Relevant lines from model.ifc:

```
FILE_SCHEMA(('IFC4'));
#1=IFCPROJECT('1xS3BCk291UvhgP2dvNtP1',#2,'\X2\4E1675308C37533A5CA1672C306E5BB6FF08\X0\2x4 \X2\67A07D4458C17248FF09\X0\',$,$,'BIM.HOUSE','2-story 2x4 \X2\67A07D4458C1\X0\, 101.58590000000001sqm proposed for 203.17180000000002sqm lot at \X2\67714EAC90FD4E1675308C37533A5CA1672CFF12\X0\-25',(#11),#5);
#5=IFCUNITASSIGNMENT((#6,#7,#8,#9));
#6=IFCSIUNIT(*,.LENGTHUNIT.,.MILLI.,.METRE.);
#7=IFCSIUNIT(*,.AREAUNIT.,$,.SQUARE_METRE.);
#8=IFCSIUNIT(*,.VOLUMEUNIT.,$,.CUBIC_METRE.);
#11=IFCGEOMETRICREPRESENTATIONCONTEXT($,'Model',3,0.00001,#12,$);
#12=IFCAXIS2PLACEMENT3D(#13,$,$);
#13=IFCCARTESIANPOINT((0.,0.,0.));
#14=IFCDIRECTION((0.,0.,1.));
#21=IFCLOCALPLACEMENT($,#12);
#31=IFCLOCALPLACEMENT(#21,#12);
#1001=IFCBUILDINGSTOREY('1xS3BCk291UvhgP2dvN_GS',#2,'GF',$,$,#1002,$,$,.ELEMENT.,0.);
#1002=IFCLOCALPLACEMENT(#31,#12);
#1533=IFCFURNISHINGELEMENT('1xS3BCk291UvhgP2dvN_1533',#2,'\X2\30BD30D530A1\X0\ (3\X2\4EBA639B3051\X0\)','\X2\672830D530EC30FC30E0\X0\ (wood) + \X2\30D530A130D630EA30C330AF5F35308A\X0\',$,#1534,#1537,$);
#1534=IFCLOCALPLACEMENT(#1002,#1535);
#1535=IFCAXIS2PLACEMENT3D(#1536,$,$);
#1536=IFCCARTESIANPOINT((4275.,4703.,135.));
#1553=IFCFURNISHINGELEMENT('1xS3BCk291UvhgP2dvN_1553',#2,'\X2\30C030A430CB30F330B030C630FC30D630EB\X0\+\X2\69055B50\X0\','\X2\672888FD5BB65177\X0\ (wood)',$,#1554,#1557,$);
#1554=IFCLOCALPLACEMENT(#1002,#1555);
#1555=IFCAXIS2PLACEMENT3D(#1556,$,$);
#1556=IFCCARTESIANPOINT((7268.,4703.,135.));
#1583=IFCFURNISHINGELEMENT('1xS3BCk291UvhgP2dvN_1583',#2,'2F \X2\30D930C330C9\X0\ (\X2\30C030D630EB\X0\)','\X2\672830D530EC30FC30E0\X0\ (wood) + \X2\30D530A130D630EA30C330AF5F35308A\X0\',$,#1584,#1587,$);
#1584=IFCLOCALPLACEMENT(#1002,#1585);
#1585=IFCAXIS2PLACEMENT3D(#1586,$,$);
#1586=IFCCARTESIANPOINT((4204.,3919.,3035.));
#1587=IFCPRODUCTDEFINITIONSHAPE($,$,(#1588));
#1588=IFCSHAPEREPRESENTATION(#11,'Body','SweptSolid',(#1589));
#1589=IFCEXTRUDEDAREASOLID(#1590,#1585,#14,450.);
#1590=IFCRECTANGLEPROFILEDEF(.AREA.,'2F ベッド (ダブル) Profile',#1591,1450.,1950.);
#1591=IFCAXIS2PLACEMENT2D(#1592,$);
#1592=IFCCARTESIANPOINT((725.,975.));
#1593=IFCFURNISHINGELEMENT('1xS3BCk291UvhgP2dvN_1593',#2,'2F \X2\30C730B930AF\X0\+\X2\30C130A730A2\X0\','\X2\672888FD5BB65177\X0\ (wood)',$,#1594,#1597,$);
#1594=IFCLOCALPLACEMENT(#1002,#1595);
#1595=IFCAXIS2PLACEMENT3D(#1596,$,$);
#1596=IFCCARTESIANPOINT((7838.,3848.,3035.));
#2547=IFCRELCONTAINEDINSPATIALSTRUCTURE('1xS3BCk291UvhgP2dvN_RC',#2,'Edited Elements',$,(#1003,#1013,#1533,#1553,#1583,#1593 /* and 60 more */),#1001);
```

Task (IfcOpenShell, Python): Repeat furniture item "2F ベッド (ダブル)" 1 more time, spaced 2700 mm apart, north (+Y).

```python
import numpy as np
import ifcopenshell
import ifcopenshell.api.geometry
import ifcopenshell.api.root
import ifcopenshell.util.element
import ifcopenshell.util.placement
import ifcopenshell.util.unit

model = ifcopenshell.open("model.ifc")
unit_scale = ifcopenshell.util.unit.calculate_unit_scale(model)


def reuse_history(source, copy):
    """copy_class also copies each property set's owner history, people and application; keep the originals."""
    for rel in copy.IsDefinedBy:
        if rel.is_a("IfcRelDefinesByProperties") and (history := rel.RelatingPropertyDefinition.OwnerHistory):
            rel.RelatingPropertyDefinition.OwnerHistory = source.OwnerHistory
            ifcopenshell.util.element.remove_deep2(model, history)


source = model.by_guid("1xS3BCk291UvhgP2dvN_1583")
base = ifcopenshell.util.placement.get_local_placement(source.ObjectPlacement)
step = np.array([0.0, 1.0, 0.0]) * 2.7 / unit_scale

for i in range(1, 2):
    copy = ifcopenshell.api.root.copy_class(model, product=source)
    copy.Representation = ifcopenshell.util.element.copy_deep(
        model, source.Representation, exclude=["IfcGeometricRepresentationContext", "IfcRepresentationMap"]
    )
    reuse_history(source, copy)
    matrix = base.copy()
    matrix[:3, 3] += i * step
    print("added at", matrix[:3, 3].round(3) + 0.0)
    ifcopenshell.api.geometry.edit_object_placement(model, product=copy, matrix=matrix, is_si=False)

model.write("model_v2.ifc")
```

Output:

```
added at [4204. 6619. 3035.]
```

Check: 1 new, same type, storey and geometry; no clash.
